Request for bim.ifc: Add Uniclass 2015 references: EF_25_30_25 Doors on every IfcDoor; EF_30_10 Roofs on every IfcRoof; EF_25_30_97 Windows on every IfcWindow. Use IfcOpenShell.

First a look at what the model holds.

```python
import ifcopenshell

model = ifcopenshell.open("bim.ifc")
print(model.schema)
print("classifications:", [c.Name for c in model.by_type("IfcClassification")])
for ifc_class in ("IfcDoor", "IfcRoof", "IfcStair", "IfcWall", "IfcWindow"):
    print(ifc_class, len(model.by_type(ifc_class)))
```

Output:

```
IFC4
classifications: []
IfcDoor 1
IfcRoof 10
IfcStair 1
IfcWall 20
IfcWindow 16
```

```python
import ifcopenshell
import ifcopenshell.api.classification

model = ifcopenshell.open("bim.ifc")

system = ifcopenshell.api.classification.add_classification(model, classification="Uniclass 2015")

codes = {
    "IfcDoor": ("EF_25_30_25", "Doors"),
    "IfcRoof": ("EF_30_10", "Roofs"),
    "IfcWindow": ("EF_25_30_97", "Windows"),
}
for ifc_class, (code, name) in codes.items():
    products = model.by_type(ifc_class)
    ifcopenshell.api.classification.add_reference(
        model, products=products, classification=system, identification=code, name=name
    )
    print(code, len(products))

model.write("bim_updated.ifc")
```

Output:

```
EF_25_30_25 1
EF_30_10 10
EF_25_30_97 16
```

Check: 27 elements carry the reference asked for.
